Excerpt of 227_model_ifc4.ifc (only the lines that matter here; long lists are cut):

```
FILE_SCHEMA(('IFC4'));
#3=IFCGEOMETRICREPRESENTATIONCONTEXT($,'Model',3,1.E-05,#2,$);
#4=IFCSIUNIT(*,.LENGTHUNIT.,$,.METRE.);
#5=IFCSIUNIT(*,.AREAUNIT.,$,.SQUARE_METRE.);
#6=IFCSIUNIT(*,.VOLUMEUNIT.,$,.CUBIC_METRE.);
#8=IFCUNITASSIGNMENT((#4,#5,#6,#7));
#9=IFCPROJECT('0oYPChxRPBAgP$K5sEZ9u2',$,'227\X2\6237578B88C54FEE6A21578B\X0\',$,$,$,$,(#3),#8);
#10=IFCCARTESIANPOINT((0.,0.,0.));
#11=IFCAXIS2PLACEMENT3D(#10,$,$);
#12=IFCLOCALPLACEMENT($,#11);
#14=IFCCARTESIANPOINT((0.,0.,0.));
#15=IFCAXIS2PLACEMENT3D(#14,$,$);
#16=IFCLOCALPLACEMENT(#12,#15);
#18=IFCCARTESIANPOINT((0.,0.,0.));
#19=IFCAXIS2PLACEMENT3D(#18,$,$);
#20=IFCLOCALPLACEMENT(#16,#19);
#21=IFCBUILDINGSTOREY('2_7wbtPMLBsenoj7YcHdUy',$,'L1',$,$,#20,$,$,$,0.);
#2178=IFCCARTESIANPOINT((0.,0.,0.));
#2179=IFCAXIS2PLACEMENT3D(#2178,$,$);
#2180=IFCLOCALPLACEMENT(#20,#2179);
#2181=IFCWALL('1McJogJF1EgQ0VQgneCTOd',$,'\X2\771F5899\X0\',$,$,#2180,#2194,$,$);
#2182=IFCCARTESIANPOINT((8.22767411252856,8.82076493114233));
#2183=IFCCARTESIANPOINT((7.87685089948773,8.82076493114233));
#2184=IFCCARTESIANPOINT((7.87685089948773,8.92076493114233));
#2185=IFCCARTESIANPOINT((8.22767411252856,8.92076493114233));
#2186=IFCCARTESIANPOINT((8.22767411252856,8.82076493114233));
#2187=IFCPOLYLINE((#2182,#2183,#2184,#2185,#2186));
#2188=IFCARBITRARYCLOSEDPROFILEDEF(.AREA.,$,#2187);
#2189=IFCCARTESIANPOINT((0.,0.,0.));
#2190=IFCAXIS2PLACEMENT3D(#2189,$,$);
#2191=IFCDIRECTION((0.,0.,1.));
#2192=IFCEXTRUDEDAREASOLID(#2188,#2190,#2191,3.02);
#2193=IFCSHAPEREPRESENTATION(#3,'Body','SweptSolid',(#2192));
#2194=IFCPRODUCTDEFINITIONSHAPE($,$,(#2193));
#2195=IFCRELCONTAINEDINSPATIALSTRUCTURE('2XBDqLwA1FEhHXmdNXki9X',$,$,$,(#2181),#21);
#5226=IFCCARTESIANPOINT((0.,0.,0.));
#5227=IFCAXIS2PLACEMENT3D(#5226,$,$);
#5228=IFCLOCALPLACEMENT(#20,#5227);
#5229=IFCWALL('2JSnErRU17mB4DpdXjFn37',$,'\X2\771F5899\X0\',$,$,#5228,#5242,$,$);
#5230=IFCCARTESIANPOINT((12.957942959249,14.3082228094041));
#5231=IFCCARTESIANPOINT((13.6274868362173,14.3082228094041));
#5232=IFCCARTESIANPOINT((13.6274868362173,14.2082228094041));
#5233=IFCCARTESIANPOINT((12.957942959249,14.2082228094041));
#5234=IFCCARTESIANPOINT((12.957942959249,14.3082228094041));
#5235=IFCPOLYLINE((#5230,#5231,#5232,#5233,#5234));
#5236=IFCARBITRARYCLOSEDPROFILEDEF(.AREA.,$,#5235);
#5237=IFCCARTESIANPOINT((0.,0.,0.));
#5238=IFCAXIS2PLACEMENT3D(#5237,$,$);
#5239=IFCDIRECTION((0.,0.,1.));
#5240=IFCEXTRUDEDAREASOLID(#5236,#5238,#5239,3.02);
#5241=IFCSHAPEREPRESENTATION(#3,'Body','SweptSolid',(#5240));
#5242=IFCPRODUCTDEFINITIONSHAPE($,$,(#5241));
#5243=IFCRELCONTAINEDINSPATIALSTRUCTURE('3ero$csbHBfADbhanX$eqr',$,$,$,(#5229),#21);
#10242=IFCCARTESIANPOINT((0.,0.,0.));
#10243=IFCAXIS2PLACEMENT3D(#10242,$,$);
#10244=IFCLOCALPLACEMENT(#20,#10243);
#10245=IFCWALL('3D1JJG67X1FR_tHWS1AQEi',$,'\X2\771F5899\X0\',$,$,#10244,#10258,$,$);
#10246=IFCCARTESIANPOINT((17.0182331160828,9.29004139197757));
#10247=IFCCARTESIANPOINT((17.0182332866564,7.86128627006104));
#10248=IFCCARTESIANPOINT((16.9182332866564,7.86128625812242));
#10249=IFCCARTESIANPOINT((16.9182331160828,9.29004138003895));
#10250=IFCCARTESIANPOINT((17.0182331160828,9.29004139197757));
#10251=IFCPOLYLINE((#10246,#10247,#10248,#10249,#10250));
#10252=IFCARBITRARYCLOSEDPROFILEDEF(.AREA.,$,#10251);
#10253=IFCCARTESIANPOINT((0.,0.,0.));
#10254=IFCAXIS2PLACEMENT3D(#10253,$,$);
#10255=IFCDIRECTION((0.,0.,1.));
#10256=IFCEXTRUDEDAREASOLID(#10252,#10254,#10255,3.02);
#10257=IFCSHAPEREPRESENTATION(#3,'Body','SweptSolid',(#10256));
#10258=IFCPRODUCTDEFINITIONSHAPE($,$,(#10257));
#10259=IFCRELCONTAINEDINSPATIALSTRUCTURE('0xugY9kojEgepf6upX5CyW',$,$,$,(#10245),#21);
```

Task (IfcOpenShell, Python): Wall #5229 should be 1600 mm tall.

```python
import ifcopenshell
import ifcopenshell.geom
import ifcopenshell.util.shape
import ifcopenshell.util.unit

model = ifcopenshell.open("227_model_ifc4.ifc")
unit_scale = ifcopenshell.util.unit.calculate_unit_scale(model)
settings = ifcopenshell.geom.settings()


def volume(element):
    """Net volume in cubic metres, openings subtracted."""
    shape = ifcopenshell.geom.create_shape(settings, element)
    return ifcopenshell.util.shape.get_volume(shape.geometry)


wall = model.by_guid("2JSnErRU17mB4DpdXjFn37")
before = volume(wall)

body = next(r for r in wall.Representation.Representations if r.RepresentationIdentifier == "Body")
solid = body.Items[0]
old_height = solid.Depth
solid.Depth = 1.6 / unit_scale
after = volume(wall)

print(f"height {old_height:g} -> {solid.Depth:g}, volume {before:.3f} -> {after:.3f} m3")

model.write("227_model_ifc4_edited.ifc")
```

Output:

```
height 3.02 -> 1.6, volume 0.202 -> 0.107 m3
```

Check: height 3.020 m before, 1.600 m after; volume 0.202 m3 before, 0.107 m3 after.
